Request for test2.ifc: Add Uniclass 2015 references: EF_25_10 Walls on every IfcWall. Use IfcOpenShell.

First a look at what the model holds.

```python
import ifcopenshell

model = ifcopenshell.open("test2.ifc")
print(model.schema)
print("classifications:", [c.Name for c in model.by_type("IfcClassification")])
for ifc_class in ("IfcDoor", "IfcRoof", "IfcStair", "IfcWall", "IfcWindow"):
    print(ifc_class, len(model.by_type(ifc_class)))
```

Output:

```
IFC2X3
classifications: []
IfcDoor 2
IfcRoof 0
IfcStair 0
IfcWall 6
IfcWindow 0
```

```python
import ifcopenshell
import ifcopenshell.api.classification

model = ifcopenshell.open("test2.ifc")

# IFC2X3 requires Source and Edition and has no link from the project to the system.
system = model.create_entity("IfcClassification", Source="NBS", Edition="2015", Name="Uniclass 2015")

codes = {
    "IfcWall": ("EF_25_10", "Walls"),
}
for ifc_class, (code, name) in codes.items():
    products = model.by_type(ifc_class)
    ifcopenshell.api.classification.add_reference(
        model, products=products, classification=system, identification=code, name=name
    )
    print(code, len(products))

model.write("test2_edited.ifc")
```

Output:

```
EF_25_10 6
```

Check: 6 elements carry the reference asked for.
